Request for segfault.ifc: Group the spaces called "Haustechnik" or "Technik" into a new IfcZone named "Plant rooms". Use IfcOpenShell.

First a look at what the model holds.

```python
import ifcopenshell

model = ifcopenshell.open("segfault.ifc")
print(model.schema)
seen = {}
for space in model.by_type("IfcSpace"):
    seen[space.LongName] = seen.get(space.LongName, 0) + 1
for name, count in sorted(seen.items(), key=str):
    print(count, "x", name)
print("zones:", [z.Name for z in model.by_type("IfcZone")][:20])
```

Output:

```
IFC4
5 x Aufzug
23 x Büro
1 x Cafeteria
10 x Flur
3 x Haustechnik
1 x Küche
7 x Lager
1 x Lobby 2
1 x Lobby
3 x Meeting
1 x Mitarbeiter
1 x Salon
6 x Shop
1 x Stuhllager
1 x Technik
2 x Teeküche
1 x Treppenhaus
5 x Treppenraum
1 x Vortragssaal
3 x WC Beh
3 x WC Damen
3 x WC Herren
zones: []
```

```python
import ifcopenshell
import ifcopenshell.api.group
import ifcopenshell.api.root

model = ifcopenshell.open("segfault.ifc")

names = {"Haustechnik", "Technik"}
spaces = [s for s in model.by_type("IfcSpace") if s.LongName in names]

zone = ifcopenshell.api.root.create_entity(model, ifc_class="IfcZone", name="Plant rooms")
ifcopenshell.api.group.assign_group(model, products=spaces, group=zone)
print(len(spaces), "spaces in", zone.Name)

model.write("segfault_v2.ifc")
```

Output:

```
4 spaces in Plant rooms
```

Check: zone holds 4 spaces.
